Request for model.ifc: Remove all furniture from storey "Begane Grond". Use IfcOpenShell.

First a look at what the model holds.

```python
import ifcopenshell
import ifcopenshell.util.element

model = ifcopenshell.open("model.ifc")
print(model.schema)
storey = next(s for s in model.by_type("IfcBuildingStorey") if s.Name == "Begane Grond")
furniture = [e for e in ifcopenshell.util.element.get_decomposition(storey) if e.is_a("IfcFurnishingElement")]
seen = {}
for e in furniture:
    element_type = ifcopenshell.util.element.get_type(e)
    name = element_type.Name if element_type not in (None, e) else None
    seen[name] = seen.get(name, 0) + 1
for name, count in sorted(seen.items(), key=str):
    print(count, "x", name)
```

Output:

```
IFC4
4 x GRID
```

```python
import ifcopenshell
import ifcopenshell.api.root
import ifcopenshell.util.element

model = ifcopenshell.open("model.ifc")

storey = next(s for s in model.by_type("IfcBuildingStorey") if s.Name == "Begane Grond")
furniture = [e for e in ifcopenshell.util.element.get_decomposition(storey) if e.is_a("IfcFurnishingElement")]

for e in furniture:
    ifcopenshell.api.root.remove_product(model, product=e)
print(len(furniture), "removed")

model.write("model_edited.ifc")
```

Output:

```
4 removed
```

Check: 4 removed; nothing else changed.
